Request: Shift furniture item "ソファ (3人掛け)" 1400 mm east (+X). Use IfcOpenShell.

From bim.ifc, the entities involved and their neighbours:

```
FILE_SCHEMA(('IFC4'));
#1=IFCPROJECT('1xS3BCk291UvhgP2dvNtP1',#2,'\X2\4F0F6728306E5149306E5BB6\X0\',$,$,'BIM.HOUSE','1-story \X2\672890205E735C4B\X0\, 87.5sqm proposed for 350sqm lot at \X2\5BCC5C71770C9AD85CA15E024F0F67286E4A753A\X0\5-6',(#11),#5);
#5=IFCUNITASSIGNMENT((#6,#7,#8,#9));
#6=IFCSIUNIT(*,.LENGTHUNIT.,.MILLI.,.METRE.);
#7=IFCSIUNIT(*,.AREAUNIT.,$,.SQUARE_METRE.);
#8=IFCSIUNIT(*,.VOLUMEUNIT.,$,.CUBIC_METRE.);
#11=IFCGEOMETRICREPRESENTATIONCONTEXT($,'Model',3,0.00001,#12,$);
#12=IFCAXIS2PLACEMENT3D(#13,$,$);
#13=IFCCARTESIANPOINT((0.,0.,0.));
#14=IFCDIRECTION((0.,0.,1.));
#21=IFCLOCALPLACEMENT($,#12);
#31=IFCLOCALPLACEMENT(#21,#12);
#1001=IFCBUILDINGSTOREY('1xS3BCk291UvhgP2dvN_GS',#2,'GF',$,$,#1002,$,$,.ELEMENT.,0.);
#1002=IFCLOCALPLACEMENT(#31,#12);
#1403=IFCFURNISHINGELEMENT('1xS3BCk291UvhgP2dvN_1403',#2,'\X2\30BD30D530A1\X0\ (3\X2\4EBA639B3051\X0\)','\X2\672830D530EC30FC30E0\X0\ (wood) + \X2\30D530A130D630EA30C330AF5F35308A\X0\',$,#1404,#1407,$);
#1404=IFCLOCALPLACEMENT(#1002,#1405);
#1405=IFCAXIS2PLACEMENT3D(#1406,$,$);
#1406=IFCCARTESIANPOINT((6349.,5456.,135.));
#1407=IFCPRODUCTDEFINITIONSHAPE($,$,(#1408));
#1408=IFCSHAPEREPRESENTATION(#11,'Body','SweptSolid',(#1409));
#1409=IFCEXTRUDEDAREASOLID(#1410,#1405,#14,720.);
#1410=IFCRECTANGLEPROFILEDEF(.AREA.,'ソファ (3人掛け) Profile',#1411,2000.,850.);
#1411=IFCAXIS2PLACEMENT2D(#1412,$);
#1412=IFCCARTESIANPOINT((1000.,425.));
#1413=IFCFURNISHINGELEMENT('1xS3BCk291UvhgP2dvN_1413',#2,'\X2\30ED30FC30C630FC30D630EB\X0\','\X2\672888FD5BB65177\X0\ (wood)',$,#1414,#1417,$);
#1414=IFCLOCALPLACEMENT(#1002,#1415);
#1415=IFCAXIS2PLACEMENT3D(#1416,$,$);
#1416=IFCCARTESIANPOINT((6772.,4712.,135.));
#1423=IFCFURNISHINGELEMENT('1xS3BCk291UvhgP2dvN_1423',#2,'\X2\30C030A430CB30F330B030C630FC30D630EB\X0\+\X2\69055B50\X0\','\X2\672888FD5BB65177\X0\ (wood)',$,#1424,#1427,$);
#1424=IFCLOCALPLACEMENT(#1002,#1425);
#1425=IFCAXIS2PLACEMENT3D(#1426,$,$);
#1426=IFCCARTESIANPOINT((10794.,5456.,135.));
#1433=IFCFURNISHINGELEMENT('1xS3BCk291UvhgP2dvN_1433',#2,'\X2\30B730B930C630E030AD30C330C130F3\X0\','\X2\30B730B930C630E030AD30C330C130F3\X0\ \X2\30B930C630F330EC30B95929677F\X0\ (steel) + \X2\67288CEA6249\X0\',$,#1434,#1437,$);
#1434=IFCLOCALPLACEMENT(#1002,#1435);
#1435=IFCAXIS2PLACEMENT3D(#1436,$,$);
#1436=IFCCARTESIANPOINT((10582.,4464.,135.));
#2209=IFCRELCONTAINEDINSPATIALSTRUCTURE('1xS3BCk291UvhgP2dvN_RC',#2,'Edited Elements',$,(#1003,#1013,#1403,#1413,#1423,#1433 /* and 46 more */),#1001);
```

```python
import ifcopenshell
import ifcopenshell.api.geometry
import ifcopenshell.util.placement
import ifcopenshell.util.unit

model = ifcopenshell.open("bim.ifc")
unit_scale = ifcopenshell.util.unit.calculate_unit_scale(model)

item = model.by_guid("1xS3BCk291UvhgP2dvN_1403")
matrix = ifcopenshell.util.placement.get_local_placement(item.ObjectPlacement)
matrix[0, 3] += 1.4 / unit_scale
ifcopenshell.api.geometry.edit_object_placement(model, product=item, matrix=matrix, is_si=False)

print(ifcopenshell.util.placement.get_local_placement(item.ObjectPlacement).round(3) + 0.0)

model.write("bim_rev.ifc")
```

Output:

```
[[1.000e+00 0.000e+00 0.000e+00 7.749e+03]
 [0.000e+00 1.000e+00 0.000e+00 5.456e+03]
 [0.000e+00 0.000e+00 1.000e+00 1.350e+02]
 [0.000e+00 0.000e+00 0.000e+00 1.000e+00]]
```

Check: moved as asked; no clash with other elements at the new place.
